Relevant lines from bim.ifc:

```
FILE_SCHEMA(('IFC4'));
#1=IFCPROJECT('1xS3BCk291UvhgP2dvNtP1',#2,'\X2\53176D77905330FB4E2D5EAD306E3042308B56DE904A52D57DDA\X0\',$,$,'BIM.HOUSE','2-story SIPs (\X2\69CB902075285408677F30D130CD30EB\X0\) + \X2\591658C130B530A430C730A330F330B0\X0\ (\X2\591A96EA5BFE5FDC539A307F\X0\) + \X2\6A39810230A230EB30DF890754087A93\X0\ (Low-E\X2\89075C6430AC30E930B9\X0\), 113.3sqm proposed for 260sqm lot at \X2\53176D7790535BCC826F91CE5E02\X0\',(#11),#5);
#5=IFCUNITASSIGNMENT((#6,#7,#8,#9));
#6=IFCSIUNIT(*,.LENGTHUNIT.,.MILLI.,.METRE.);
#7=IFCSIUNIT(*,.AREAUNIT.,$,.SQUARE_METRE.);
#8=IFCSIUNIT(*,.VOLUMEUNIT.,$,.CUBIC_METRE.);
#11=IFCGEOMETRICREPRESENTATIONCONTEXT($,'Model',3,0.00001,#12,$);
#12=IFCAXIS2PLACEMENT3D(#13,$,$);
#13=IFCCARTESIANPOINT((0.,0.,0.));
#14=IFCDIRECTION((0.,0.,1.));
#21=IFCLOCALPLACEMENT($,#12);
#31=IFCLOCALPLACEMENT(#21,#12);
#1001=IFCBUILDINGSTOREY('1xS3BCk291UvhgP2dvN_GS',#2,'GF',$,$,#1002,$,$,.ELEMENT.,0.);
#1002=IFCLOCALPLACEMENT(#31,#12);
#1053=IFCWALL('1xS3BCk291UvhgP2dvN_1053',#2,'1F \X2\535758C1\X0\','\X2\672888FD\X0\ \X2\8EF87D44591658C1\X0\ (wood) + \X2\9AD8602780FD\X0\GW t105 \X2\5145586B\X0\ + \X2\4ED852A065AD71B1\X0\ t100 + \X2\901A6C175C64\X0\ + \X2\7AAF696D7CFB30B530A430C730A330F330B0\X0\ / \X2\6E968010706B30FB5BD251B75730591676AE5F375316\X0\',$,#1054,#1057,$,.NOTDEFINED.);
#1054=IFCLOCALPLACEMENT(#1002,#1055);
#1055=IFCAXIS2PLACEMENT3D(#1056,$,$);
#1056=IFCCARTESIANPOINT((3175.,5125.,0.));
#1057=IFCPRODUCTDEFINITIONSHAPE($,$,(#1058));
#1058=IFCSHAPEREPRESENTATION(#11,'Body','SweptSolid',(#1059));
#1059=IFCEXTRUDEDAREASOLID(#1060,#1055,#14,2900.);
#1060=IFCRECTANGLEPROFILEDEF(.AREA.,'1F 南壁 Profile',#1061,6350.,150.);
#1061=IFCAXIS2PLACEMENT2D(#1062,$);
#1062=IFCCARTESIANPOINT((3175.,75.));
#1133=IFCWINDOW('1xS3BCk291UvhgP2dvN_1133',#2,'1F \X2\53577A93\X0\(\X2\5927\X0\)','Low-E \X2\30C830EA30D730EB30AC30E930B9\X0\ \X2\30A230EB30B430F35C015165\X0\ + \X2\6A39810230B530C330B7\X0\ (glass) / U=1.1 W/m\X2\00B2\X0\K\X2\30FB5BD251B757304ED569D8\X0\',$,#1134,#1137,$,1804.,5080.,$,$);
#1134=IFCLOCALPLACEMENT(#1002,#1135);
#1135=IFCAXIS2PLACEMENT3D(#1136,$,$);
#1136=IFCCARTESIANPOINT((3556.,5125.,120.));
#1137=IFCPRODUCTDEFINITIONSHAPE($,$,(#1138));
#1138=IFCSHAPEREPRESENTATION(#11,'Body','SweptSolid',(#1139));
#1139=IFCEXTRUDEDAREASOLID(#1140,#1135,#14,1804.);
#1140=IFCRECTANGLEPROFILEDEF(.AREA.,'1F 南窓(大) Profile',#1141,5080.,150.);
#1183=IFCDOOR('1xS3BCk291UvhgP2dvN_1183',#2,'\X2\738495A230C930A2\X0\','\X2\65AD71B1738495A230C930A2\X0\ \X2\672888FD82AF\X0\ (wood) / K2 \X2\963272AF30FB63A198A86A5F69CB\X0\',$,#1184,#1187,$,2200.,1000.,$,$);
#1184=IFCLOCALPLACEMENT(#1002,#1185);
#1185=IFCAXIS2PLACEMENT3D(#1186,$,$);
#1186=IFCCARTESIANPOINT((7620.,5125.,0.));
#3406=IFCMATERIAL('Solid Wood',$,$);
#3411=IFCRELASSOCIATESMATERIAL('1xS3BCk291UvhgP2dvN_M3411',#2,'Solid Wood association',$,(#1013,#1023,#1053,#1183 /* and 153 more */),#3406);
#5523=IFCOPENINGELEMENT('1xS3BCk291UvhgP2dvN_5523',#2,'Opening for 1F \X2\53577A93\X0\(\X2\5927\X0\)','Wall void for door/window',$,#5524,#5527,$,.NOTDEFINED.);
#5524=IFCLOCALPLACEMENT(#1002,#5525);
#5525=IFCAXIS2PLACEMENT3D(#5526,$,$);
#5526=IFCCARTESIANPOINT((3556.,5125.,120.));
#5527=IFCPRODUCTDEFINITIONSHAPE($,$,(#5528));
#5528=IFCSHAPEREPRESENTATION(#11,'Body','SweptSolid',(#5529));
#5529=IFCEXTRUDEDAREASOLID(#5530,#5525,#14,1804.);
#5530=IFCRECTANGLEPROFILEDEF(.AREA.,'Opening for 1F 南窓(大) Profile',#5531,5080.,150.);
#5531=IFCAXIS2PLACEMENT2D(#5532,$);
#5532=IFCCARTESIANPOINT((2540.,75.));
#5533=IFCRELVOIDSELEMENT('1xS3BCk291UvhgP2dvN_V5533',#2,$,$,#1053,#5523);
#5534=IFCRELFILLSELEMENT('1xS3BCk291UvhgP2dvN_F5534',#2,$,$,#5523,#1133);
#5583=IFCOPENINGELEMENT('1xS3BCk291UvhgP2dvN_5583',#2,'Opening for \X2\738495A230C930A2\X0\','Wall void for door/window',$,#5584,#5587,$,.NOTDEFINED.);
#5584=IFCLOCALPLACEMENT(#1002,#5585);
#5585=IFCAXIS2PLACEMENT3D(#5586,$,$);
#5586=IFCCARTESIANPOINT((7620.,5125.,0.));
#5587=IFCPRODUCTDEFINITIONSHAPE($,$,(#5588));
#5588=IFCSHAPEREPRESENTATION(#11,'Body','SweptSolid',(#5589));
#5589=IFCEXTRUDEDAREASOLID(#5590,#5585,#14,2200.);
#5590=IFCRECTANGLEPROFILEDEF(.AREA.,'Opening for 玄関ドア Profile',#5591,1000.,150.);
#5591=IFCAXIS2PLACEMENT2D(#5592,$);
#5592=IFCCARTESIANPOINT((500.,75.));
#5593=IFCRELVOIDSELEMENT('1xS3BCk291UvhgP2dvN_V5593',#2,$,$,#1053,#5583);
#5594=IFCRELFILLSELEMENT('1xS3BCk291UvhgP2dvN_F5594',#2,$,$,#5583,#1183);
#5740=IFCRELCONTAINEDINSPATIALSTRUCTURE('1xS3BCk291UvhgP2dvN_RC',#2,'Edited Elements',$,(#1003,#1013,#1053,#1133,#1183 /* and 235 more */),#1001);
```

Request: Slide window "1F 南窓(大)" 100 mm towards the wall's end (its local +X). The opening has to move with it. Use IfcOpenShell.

```python
import ifcopenshell
import ifcopenshell.api.geometry
import ifcopenshell.util.placement

model = ifcopenshell.open("bim.ifc")

window = model.by_id(1133)
opening = window.FillsVoids[0].RelatingOpeningElement
wall = opening.VoidsElements[0].RelatingBuildingElement

wall_matrix = ifcopenshell.util.placement.get_local_placement(wall.ObjectPlacement)
shift = wall_matrix[:3, 0] * 100.0
before = ifcopenshell.util.placement.get_local_placement(window.ObjectPlacement)[:3, 3].copy()

# The window is not placed relative to its opening, so move both.
for product in (opening, window):
    matrix = ifcopenshell.util.placement.get_local_placement(product.ObjectPlacement)
    matrix[:3, 3] += shift
    ifcopenshell.api.geometry.edit_object_placement(model, product=product, matrix=matrix, is_si=False)

after = ifcopenshell.util.placement.get_local_placement(window.ObjectPlacement)[:3, 3]
print("window moved by", (after - before).round(3) + 0.0)

model.write("bim_rev.ifc")
```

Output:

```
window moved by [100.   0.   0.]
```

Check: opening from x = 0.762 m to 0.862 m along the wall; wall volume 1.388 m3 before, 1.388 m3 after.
